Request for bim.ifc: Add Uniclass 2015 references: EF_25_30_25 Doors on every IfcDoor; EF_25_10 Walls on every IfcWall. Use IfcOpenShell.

First a look at what the model holds.

```python
import ifcopenshell

model = ifcopenshell.open("bim.ifc")
print(model.schema)
print("classifications:", [c.Name for c in model.by_type("IfcClassification")])
for ifc_class in ("IfcDoor", "IfcRoof", "IfcStair", "IfcWall", "IfcWindow"):
    print(ifc_class, len(model.by_type(ifc_class)))
```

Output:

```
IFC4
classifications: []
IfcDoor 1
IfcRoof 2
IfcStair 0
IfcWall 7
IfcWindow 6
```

```python
import ifcopenshell
import ifcopenshell.api.classification

model = ifcopenshell.open("bim.ifc")

system = ifcopenshell.api.classification.add_classification(model, classification="Uniclass 2015")

codes = {
    "IfcDoor": ("EF_25_30_25", "Doors"),
    "IfcWall": ("EF_25_10", "Walls"),
}
for ifc_class, (code, name) in codes.items():
    products = model.by_type(ifc_class)
    ifcopenshell.api.classification.add_reference(
        model, products=products, classification=system, identification=code, name=name
    )
    print(code, len(products))

model.write("bim-out.ifc")
```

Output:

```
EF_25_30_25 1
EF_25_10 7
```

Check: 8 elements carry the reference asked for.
